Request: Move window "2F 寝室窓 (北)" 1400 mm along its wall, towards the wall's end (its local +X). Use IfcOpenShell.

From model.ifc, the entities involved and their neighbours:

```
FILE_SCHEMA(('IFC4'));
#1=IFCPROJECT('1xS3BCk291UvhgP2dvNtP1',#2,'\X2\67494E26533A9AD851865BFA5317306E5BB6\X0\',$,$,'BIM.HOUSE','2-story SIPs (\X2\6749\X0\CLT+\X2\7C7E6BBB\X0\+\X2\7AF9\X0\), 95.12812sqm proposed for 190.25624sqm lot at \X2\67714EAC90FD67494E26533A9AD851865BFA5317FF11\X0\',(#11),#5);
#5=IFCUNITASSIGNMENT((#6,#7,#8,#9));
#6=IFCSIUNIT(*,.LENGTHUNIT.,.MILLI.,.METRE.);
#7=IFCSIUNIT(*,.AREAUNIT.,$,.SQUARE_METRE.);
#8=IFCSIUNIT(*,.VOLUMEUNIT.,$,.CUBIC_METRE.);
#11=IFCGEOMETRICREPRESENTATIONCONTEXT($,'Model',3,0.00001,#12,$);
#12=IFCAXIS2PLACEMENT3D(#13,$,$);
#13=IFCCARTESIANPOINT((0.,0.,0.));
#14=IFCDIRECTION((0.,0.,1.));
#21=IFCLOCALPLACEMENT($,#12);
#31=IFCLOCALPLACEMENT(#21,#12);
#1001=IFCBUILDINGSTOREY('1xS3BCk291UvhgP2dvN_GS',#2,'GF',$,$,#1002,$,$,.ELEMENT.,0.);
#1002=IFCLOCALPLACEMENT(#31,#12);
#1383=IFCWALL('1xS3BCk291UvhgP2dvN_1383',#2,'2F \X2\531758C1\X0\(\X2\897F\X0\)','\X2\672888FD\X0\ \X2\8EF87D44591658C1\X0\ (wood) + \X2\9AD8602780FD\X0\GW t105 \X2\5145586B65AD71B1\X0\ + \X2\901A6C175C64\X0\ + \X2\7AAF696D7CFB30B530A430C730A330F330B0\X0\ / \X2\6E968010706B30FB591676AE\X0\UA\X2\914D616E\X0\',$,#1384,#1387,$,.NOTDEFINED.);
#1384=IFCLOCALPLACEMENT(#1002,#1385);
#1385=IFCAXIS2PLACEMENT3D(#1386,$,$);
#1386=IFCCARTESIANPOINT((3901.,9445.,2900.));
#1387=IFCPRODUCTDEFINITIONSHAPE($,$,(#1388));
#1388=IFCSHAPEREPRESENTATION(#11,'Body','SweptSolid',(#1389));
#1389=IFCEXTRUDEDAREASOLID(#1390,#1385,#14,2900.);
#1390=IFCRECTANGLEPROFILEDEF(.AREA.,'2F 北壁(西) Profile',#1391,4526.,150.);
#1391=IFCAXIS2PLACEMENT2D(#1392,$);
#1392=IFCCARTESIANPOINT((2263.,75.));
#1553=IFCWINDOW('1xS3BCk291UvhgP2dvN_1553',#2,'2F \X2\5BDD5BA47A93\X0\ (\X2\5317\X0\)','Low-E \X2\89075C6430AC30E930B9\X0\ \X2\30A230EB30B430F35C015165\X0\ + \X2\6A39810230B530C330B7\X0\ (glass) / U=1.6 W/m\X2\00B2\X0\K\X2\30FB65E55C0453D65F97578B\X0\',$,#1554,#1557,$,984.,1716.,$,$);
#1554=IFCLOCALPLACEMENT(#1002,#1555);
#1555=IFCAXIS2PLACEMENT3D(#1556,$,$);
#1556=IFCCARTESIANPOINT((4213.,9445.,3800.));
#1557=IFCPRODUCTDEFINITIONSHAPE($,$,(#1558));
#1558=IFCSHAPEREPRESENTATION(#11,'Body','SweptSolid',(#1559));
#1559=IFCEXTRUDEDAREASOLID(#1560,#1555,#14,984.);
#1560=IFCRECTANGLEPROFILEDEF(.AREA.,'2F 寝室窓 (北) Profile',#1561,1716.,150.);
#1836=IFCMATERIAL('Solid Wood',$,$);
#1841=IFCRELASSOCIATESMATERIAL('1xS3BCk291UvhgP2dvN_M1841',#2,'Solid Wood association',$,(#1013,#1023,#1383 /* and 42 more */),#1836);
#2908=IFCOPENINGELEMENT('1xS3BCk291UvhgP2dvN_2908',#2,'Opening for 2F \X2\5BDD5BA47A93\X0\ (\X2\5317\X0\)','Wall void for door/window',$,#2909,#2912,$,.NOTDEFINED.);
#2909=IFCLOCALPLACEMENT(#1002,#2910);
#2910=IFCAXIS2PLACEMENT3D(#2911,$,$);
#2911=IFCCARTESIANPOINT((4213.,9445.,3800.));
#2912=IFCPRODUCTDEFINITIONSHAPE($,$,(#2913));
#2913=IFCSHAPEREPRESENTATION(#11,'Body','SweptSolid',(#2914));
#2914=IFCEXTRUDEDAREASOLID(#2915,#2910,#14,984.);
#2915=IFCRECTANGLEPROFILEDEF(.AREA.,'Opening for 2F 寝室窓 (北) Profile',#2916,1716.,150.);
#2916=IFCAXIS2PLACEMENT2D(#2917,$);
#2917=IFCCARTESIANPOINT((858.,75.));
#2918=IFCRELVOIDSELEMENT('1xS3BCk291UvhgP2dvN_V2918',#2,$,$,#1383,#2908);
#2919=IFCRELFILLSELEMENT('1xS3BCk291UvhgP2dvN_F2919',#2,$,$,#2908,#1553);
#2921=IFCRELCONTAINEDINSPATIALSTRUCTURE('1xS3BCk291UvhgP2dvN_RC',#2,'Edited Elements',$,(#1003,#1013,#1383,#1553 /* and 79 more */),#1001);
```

```python
import ifcopenshell
import ifcopenshell.api.geometry
import ifcopenshell.util.placement

model = ifcopenshell.open("model.ifc")

window = model.by_id(1553)
opening = window.FillsVoids[0].RelatingOpeningElement
wall = opening.VoidsElements[0].RelatingBuildingElement

wall_matrix = ifcopenshell.util.placement.get_local_placement(wall.ObjectPlacement)
shift = wall_matrix[:3, 0] * 1400.0
before = ifcopenshell.util.placement.get_local_placement(window.ObjectPlacement)[:3, 3].copy()

# The window is not placed relative to its opening, so move both.
for product in (opening, window):
    matrix = ifcopenshell.util.placement.get_local_placement(product.ObjectPlacement)
    matrix[:3, 3] += shift
    ifcopenshell.api.geometry.edit_object_placement(model, product=product, matrix=matrix, is_si=False)

after = ifcopenshell.util.placement.get_local_placement(window.ObjectPlacement)[:3, 3]
print("window moved by", (after - before).round(3) + 0.0)

model.write("model_updated.ifc")
```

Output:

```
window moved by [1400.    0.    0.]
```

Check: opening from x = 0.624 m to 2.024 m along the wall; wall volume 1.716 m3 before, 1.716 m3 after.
